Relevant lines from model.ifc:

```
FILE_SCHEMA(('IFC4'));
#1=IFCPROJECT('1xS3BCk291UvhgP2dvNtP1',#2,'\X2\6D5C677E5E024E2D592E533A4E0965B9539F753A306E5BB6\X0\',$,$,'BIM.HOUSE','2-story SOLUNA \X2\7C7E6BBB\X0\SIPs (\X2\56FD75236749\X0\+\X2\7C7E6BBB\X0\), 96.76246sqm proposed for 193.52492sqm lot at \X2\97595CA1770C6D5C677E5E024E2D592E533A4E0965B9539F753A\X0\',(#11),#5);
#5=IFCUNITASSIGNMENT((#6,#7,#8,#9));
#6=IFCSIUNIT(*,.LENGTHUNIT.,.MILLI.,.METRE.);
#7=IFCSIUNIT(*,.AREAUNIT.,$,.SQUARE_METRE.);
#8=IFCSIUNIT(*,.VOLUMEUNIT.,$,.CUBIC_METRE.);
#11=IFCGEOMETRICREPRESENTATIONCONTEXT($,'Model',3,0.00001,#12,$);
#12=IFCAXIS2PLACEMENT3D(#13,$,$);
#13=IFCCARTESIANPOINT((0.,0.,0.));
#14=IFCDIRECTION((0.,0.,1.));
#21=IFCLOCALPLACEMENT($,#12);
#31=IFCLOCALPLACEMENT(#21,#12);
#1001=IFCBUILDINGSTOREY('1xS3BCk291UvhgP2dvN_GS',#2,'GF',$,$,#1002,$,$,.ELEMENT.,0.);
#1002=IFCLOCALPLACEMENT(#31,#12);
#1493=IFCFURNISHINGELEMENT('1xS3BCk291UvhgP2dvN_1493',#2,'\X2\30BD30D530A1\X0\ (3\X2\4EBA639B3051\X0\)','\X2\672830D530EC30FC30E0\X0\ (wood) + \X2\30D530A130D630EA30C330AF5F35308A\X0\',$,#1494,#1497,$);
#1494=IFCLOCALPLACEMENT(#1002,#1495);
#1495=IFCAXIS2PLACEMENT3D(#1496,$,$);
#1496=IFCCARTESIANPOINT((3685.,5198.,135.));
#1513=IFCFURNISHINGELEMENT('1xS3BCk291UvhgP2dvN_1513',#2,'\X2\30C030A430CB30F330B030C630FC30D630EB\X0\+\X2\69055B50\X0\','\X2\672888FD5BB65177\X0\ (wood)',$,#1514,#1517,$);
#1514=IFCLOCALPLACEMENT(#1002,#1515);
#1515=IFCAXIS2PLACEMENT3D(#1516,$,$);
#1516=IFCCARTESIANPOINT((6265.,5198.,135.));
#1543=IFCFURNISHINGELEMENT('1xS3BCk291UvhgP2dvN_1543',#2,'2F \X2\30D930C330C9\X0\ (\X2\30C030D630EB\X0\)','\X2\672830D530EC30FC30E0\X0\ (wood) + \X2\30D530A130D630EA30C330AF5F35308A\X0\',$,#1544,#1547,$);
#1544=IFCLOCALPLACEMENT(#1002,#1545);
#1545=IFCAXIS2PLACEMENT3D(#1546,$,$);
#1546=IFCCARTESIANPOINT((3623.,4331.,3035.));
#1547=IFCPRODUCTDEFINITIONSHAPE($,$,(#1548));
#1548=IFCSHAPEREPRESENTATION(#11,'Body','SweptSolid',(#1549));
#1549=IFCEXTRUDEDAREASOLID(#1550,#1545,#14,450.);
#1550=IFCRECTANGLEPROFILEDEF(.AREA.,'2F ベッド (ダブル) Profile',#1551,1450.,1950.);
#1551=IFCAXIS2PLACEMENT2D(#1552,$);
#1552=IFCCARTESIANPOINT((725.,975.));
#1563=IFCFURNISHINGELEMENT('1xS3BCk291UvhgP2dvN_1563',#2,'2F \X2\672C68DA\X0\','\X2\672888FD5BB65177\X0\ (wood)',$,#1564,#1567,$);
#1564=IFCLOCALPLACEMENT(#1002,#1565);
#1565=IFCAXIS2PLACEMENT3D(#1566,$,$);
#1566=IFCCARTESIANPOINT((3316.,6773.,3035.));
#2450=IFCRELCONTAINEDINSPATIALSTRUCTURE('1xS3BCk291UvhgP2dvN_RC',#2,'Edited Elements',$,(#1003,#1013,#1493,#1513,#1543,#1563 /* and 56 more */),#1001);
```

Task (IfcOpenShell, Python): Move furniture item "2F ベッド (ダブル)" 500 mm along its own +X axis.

```python
import ifcopenshell
import ifcopenshell.api.geometry
import ifcopenshell.util.placement
import ifcopenshell.util.unit

model = ifcopenshell.open("model.ifc")
unit_scale = ifcopenshell.util.unit.calculate_unit_scale(model)

item = model.by_guid("1xS3BCk291UvhgP2dvN_1543")
matrix = ifcopenshell.util.placement.get_local_placement(item.ObjectPlacement)
matrix[:3, 3] += matrix[:3, 0] * 0.5 / unit_scale
ifcopenshell.api.geometry.edit_object_placement(model, product=item, matrix=matrix, is_si=False)

print(ifcopenshell.util.placement.get_local_placement(item.ObjectPlacement).round(3) + 0.0)

model.write("model_updated.ifc")
```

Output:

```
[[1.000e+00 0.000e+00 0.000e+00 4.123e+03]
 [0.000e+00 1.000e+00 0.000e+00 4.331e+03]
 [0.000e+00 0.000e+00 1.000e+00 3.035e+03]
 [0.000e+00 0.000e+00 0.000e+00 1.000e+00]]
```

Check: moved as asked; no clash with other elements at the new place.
